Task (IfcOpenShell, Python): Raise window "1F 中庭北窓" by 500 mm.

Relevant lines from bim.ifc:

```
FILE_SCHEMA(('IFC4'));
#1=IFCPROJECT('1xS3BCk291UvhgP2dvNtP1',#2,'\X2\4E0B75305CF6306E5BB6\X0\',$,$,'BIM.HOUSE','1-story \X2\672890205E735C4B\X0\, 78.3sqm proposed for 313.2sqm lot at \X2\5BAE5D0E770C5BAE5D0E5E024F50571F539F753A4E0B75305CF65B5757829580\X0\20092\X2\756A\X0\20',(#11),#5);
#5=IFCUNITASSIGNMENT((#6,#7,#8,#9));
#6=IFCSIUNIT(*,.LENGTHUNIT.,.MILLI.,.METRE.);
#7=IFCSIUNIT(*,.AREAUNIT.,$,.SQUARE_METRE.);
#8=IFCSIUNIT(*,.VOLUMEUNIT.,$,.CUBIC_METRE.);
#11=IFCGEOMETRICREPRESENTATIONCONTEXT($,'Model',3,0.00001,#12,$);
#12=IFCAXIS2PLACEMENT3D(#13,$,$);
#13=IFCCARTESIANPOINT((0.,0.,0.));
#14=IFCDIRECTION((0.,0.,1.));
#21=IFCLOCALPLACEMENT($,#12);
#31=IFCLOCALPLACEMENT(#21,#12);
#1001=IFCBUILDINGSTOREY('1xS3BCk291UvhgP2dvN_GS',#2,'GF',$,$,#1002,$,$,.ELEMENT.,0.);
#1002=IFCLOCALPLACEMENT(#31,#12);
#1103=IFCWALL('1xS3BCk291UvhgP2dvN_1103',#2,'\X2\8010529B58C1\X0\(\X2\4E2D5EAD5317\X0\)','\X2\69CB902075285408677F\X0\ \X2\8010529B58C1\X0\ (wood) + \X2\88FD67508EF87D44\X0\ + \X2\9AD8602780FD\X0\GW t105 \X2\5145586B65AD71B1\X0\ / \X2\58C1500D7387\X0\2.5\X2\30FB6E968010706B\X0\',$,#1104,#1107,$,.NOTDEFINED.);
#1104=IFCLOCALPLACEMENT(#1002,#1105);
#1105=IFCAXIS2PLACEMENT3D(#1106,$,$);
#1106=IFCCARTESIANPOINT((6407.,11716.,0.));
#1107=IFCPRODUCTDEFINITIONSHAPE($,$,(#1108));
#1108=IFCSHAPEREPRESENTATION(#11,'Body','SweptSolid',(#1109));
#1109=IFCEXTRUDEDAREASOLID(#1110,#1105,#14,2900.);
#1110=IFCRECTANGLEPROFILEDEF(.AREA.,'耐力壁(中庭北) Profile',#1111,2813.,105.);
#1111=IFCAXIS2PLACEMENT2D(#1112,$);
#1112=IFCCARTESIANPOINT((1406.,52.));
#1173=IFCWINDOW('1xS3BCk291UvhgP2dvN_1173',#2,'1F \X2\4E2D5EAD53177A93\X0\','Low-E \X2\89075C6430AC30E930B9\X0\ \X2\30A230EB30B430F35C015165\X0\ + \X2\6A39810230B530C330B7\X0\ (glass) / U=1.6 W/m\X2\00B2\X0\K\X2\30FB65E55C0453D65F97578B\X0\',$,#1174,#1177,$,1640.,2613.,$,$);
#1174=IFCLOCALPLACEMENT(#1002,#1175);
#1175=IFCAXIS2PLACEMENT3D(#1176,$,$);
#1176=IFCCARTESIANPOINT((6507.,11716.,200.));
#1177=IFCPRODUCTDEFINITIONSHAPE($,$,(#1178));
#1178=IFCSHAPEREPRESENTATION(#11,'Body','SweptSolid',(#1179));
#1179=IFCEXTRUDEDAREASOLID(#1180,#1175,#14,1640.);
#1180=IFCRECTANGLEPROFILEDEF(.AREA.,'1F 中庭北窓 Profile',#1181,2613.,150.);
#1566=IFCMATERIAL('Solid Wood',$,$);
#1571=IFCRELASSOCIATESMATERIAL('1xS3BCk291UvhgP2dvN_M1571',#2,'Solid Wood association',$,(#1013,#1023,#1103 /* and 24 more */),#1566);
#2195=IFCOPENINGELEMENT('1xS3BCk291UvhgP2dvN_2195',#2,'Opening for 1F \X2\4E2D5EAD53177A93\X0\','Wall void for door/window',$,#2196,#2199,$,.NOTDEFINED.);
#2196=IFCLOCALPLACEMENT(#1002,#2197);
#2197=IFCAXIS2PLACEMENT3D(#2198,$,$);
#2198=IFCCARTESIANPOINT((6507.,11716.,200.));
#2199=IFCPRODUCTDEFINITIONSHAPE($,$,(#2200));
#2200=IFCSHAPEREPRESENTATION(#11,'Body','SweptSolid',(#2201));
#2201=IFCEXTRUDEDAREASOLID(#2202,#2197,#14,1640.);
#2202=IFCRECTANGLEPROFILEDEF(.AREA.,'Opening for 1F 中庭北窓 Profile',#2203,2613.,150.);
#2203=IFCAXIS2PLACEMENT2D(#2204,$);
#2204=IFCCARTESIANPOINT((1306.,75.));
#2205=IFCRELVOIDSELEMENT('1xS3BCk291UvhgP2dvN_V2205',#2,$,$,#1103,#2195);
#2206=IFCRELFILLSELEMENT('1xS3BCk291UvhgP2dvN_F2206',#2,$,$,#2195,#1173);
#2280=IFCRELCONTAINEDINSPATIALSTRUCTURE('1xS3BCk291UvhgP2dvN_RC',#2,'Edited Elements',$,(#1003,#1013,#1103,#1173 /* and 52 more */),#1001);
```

```python
import numpy as np
import ifcopenshell
import ifcopenshell.api.geometry
import ifcopenshell.util.placement
import ifcopenshell.util.unit

model = ifcopenshell.open("bim.ifc")
unit_scale = ifcopenshell.util.unit.calculate_unit_scale(model)

window = model.by_guid("1xS3BCk291UvhgP2dvN_1173")
opening = window.FillsVoids[0].RelatingOpeningElement
dz = 0.5 / unit_scale

shift = np.array([0.0, 0.0, dz])
# The window is not placed relative to its opening, so move both.
for product in (opening, window):
    matrix = ifcopenshell.util.placement.get_local_placement(product.ObjectPlacement)
    matrix[:3, 3] += shift
    ifcopenshell.api.geometry.edit_object_placement(model, product=product, matrix=matrix, is_si=False)

print(f"moved by {dz * unit_scale:+.3f} m")

model.write("bim_v2.ifc")
```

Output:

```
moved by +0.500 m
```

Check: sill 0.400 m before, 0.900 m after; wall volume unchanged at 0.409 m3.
